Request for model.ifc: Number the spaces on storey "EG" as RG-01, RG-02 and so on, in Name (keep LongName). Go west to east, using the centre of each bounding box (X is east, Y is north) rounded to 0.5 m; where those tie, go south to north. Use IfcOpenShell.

First a look at what the model holds.

```python
import ifcopenshell
import ifcopenshell.util.element
import ifcopenshell.util.placement

model = ifcopenshell.open("model.ifc")
print(model.schema)
storey = next(s for s in model.by_type("IfcBuildingStorey") if s.Name == "EG")
spaces = [e for e in ifcopenshell.util.element.get_decomposition(storey) if e.is_a("IfcSpace")]
for e in sorted(spaces, key=lambda e: e.id()):
    origin = ifcopenshell.util.placement.get_local_placement(e.ObjectPlacement)[:3, 3]
    print(e.id(), e.Name, e.LongName, origin.round(2) + 0.0, sep=" | ")
```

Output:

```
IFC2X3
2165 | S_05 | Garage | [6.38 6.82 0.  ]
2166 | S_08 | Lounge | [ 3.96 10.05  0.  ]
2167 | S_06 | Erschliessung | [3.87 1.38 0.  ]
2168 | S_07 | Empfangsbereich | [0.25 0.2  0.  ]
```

```python
import ifcopenshell
import ifcopenshell.geom
import ifcopenshell.util.element
import ifcopenshell.util.shape

model = ifcopenshell.open("model.ifc")
settings = ifcopenshell.geom.settings()
settings.set("use-world-coords", True)


def centre(element):
    shape = ifcopenshell.geom.create_shape(settings, element)
    return ifcopenshell.util.shape.get_bbox_centroid(shape.geometry)


storey = next(s for s in model.by_type("IfcBuildingStorey") if s.Name == "EG")
spaces = [e for e in ifcopenshell.util.element.get_decomposition(storey) if e.is_a("IfcSpace")]

# Insertion points can sit at a corner or the storey origin, so sort by the geometry (in metres).
centres = {e: centre(e) for e in spaces}
spaces.sort(key=lambda e: (round(centres[e][0] / 0.5), centres[e][1]))

for i, e in enumerate(spaces, start=1):
    number = f"RG-{i:02d}"
    e.Name = number
    print(e.id(), number)

model.write("model_edited.ifc")
```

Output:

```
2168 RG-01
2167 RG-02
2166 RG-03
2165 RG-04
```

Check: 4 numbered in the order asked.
